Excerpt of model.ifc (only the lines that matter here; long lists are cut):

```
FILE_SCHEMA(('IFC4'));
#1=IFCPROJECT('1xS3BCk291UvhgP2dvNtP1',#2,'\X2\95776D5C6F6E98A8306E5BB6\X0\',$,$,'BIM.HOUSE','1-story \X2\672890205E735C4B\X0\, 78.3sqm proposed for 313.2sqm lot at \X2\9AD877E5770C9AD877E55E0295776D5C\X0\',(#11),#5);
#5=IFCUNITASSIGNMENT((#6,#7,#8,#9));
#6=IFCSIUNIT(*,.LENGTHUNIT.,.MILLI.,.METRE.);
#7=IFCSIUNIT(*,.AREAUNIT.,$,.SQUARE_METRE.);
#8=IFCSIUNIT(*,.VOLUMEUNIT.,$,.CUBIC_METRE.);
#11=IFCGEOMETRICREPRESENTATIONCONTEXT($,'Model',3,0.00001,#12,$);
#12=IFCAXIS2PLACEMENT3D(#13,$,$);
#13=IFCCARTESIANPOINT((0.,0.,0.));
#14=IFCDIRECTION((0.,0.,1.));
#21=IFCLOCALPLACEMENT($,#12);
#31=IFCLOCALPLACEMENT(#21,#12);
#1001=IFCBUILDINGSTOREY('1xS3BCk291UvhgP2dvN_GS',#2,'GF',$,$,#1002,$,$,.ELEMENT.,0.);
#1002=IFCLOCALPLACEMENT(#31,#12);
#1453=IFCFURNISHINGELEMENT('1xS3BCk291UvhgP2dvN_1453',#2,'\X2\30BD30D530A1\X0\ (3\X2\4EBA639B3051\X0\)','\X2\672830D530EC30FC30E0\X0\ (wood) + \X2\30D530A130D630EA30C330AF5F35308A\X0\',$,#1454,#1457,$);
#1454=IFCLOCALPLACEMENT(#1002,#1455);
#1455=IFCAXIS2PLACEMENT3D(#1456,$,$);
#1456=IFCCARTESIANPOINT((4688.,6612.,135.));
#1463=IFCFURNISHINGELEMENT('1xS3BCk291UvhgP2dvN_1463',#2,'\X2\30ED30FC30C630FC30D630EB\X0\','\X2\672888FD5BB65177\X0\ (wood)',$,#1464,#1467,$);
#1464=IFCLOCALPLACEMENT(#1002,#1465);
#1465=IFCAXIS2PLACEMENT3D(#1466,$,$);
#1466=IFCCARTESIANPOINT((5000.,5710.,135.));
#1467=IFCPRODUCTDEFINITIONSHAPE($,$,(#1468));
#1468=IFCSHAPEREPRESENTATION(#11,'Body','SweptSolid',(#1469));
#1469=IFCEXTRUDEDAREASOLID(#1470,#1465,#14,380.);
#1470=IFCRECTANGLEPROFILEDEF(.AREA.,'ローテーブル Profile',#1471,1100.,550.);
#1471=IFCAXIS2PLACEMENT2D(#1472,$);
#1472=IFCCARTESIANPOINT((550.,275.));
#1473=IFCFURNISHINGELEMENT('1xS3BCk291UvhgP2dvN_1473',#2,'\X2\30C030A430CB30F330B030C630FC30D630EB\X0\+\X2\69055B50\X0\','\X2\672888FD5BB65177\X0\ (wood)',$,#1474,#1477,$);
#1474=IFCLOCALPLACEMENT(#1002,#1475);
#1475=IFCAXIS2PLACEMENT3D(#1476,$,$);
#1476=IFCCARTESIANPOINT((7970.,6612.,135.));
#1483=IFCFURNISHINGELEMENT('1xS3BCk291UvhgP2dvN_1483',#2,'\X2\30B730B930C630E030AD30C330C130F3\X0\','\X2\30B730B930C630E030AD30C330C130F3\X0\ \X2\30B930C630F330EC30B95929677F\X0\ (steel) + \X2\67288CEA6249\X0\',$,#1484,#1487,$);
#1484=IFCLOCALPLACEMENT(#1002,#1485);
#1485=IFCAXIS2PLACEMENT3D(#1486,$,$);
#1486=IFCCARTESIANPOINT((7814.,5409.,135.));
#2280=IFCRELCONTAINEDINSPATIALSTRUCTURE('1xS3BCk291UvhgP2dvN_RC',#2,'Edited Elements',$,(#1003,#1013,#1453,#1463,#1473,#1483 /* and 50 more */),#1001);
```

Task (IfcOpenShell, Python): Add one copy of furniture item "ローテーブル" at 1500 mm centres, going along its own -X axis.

```python
import ifcopenshell
import ifcopenshell.api.geometry
import ifcopenshell.api.root
import ifcopenshell.util.element
import ifcopenshell.util.placement
import ifcopenshell.util.unit

model = ifcopenshell.open("model.ifc")
unit_scale = ifcopenshell.util.unit.calculate_unit_scale(model)


def reuse_history(source, copy):
    """copy_class also copies each property set's owner history, people and application; keep the originals."""
    for rel in copy.IsDefinedBy:
        if rel.is_a("IfcRelDefinesByProperties") and (history := rel.RelatingPropertyDefinition.OwnerHistory):
            rel.RelatingPropertyDefinition.OwnerHistory = source.OwnerHistory
            ifcopenshell.util.element.remove_deep2(model, history)


source = model.by_guid("1xS3BCk291UvhgP2dvN_1463")
base = ifcopenshell.util.placement.get_local_placement(source.ObjectPlacement)
step = -base[:3, 0] * 1.5 / unit_scale

for i in range(1, 2):
    copy = ifcopenshell.api.root.copy_class(model, product=source)
    copy.Representation = ifcopenshell.util.element.copy_deep(
        model, source.Representation, exclude=["IfcGeometricRepresentationContext", "IfcRepresentationMap"]
    )
    reuse_history(source, copy)
    matrix = base.copy()
    matrix[:3, 3] += i * step
    print("added at", matrix[:3, 3].round(3) + 0.0)
    ifcopenshell.api.geometry.edit_object_placement(model, product=copy, matrix=matrix, is_si=False)

model.write("model_edited.ifc")
```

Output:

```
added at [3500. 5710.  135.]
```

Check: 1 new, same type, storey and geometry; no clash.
